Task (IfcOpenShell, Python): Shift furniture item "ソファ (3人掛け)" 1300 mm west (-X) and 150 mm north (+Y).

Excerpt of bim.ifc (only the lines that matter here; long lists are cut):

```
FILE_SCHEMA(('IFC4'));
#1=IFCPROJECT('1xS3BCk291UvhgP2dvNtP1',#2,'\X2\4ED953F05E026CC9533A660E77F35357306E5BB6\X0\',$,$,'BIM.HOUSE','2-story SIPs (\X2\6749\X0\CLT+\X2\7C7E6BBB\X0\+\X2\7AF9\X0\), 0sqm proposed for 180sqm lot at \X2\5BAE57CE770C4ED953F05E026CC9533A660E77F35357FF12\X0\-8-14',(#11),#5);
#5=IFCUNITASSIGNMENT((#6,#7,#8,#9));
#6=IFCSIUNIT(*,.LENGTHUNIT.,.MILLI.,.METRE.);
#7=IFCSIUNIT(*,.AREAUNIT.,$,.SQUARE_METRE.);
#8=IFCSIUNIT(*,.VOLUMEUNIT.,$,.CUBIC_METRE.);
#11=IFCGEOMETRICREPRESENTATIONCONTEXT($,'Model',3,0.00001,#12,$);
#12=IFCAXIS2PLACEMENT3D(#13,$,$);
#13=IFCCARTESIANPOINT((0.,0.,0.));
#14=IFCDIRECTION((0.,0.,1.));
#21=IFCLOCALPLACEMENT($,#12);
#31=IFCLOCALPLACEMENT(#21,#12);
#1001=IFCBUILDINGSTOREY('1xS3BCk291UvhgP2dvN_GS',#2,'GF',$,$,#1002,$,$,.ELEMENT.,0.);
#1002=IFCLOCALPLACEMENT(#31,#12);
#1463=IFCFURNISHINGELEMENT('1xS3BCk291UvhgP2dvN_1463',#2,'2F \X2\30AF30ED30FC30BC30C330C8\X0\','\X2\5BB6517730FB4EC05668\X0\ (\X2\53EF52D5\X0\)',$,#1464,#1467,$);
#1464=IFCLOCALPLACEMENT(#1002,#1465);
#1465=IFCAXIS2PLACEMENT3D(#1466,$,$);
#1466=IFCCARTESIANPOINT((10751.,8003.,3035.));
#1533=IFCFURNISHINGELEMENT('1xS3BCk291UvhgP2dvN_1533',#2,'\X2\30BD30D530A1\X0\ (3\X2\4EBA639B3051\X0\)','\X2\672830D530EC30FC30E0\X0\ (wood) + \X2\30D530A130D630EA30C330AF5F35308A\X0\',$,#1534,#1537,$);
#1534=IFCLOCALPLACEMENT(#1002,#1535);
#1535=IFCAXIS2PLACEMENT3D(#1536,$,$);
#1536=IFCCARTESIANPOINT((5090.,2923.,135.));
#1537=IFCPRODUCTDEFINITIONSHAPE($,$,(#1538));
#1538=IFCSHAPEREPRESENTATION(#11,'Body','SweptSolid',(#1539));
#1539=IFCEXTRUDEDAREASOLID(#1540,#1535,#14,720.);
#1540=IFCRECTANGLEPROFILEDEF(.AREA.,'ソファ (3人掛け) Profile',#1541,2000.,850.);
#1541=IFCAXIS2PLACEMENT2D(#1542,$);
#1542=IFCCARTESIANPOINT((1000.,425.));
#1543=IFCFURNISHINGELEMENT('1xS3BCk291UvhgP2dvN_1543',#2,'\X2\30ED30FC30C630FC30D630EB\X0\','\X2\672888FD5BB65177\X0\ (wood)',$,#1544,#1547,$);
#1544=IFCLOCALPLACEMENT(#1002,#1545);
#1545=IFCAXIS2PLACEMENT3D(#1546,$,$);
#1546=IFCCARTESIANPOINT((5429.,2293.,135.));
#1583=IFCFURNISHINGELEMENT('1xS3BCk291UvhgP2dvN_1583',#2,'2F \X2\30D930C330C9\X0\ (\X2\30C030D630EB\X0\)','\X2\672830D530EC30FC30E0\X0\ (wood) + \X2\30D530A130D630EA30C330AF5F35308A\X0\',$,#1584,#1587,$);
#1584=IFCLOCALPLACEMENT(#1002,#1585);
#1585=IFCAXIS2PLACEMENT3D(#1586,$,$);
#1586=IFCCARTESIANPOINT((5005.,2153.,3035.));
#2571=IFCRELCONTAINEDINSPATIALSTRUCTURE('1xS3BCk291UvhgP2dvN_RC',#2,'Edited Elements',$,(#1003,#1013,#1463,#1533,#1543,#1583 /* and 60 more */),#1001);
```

```python
import ifcopenshell
import ifcopenshell.api.geometry
import ifcopenshell.util.placement
import ifcopenshell.util.unit

model = ifcopenshell.open("bim.ifc")
unit_scale = ifcopenshell.util.unit.calculate_unit_scale(model)

item = model.by_guid("1xS3BCk291UvhgP2dvN_1533")
matrix = ifcopenshell.util.placement.get_local_placement(item.ObjectPlacement)
matrix[0, 3] -= 1.3 / unit_scale
matrix[1, 3] += 0.15 / unit_scale
ifcopenshell.api.geometry.edit_object_placement(model, product=item, matrix=matrix, is_si=False)

print(ifcopenshell.util.placement.get_local_placement(item.ObjectPlacement).round(3) + 0.0)

model.write("bim_updated.ifc")
```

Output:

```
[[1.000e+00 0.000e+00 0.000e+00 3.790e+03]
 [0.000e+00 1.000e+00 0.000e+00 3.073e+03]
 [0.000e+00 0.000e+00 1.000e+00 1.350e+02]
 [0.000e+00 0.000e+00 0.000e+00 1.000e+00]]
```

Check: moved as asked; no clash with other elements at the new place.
